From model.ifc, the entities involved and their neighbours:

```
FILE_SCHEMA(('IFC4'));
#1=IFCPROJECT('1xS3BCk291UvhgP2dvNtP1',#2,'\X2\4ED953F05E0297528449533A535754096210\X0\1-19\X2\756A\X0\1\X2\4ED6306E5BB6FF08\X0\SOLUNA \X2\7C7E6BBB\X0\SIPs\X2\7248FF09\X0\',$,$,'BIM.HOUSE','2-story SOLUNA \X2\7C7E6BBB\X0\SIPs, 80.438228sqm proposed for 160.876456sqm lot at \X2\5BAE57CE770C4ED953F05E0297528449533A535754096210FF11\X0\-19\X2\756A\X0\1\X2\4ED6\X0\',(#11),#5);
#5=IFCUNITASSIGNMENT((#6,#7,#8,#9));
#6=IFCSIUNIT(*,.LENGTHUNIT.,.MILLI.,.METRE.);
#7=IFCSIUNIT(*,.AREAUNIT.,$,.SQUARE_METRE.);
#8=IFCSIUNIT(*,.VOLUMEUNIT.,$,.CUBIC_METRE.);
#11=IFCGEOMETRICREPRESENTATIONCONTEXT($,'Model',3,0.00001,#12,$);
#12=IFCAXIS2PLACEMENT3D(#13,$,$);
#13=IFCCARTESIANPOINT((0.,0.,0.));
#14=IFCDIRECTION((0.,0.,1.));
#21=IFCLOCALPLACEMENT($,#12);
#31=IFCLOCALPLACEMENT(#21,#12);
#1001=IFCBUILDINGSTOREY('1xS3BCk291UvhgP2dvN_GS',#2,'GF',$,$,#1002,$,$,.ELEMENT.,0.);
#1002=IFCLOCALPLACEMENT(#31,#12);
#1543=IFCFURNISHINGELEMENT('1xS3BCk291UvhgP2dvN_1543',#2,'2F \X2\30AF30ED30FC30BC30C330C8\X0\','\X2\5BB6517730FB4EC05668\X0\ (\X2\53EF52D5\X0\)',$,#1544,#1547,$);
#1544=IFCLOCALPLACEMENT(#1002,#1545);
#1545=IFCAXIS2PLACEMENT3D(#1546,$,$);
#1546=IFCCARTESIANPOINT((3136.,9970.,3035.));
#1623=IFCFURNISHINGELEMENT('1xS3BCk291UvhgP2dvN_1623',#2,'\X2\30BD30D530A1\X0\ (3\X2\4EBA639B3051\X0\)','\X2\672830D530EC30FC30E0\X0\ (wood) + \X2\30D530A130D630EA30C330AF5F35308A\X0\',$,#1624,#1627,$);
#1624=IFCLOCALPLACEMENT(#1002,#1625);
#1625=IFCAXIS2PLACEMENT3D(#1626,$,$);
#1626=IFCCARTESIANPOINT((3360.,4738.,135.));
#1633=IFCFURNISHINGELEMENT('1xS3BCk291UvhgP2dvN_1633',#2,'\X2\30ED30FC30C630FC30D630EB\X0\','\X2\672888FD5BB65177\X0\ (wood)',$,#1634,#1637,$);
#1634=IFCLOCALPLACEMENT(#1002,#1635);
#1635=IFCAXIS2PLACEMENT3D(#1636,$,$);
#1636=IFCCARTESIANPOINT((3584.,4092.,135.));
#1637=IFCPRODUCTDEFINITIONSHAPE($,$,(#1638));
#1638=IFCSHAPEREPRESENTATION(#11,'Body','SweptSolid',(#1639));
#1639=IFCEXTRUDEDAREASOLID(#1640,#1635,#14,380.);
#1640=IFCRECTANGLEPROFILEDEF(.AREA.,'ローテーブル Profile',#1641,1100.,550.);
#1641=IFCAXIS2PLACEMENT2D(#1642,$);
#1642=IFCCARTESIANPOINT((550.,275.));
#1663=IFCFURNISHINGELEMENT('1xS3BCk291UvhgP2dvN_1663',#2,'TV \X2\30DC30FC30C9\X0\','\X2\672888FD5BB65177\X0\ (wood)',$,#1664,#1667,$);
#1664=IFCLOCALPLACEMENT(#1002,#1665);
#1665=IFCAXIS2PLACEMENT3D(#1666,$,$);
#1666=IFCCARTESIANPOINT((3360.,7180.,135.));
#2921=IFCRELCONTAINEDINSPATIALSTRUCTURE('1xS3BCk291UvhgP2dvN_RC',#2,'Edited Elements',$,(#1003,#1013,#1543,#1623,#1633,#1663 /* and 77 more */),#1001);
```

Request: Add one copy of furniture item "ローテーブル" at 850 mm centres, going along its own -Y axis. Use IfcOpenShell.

```python
import ifcopenshell
import ifcopenshell.api.geometry
import ifcopenshell.api.root
import ifcopenshell.util.element
import ifcopenshell.util.placement

model = ifcopenshell.open("model.ifc")


def reuse_history(source, copy):
    """copy_class also copies each property set's owner history, people and application; keep the originals."""
    for rel in copy.IsDefinedBy:
        if rel.is_a("IfcRelDefinesByProperties") and (history := rel.RelatingPropertyDefinition.OwnerHistory):
            rel.RelatingPropertyDefinition.OwnerHistory = source.OwnerHistory
            ifcopenshell.util.element.remove_deep2(model, history)


source = model.by_id(1633)
base = ifcopenshell.util.placement.get_local_placement(source.ObjectPlacement)
step = -base[:3, 1] * 850.0

for i in range(1, 2):
    copy = ifcopenshell.api.root.copy_class(model, product=source)
    copy.Representation = ifcopenshell.util.element.copy_deep(
        model, source.Representation, exclude=["IfcGeometricRepresentationContext", "IfcRepresentationMap"]
    )
    reuse_history(source, copy)
    matrix = base.copy()
    matrix[:3, 3] += i * step
    print("added at", matrix[:3, 3].round(3) + 0.0)
    ifcopenshell.api.geometry.edit_object_placement(model, product=copy, matrix=matrix, is_si=False)

model.write("model-out.ifc")
```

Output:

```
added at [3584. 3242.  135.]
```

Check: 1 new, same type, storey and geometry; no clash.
